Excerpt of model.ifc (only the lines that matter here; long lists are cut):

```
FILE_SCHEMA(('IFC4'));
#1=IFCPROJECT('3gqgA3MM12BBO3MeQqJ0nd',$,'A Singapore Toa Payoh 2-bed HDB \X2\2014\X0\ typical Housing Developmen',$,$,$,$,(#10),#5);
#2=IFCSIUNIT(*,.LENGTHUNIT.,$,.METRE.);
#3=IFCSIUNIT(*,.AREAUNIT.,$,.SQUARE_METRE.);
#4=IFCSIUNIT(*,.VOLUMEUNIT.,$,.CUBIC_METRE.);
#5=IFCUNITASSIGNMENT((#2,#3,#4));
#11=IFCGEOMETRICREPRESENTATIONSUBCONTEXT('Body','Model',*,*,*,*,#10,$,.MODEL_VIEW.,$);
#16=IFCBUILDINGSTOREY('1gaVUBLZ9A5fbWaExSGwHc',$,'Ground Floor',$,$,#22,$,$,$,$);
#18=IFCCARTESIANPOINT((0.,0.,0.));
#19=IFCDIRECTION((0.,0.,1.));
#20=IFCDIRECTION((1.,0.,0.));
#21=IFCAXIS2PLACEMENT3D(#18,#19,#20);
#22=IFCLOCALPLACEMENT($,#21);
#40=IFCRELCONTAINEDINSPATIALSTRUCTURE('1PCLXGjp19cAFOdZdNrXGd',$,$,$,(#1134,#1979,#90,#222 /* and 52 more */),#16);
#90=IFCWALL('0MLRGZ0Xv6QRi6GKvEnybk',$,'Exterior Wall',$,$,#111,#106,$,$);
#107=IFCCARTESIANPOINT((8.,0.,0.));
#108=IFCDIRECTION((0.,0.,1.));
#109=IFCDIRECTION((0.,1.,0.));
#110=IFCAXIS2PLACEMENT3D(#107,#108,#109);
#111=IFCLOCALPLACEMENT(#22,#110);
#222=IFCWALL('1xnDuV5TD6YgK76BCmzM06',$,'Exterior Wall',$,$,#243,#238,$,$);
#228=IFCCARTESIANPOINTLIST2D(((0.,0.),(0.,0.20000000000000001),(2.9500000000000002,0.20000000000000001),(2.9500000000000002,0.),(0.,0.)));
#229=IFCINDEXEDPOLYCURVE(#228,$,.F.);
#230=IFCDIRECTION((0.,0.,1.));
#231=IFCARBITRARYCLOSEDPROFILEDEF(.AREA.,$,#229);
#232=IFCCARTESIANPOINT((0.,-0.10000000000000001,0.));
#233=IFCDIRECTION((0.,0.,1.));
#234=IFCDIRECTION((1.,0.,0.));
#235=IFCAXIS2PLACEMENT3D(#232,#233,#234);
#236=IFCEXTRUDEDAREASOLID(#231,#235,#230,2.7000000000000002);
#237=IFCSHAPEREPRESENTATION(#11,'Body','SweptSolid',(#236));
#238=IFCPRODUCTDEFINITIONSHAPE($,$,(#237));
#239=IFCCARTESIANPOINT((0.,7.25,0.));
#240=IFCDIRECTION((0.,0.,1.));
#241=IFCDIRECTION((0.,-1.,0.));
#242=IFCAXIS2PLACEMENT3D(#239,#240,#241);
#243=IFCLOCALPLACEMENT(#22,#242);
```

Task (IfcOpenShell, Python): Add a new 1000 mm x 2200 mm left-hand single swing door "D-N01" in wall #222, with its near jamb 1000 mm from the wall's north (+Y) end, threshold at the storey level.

```python
import numpy as np
import ifcopenshell
import ifcopenshell.api.feature
import ifcopenshell.api.geometry
import ifcopenshell.api.root
import ifcopenshell.api.spatial
import ifcopenshell.geom
import ifcopenshell.util.element
import ifcopenshell.util.placement
import ifcopenshell.util.representation
import ifcopenshell.util.shape
import ifcopenshell.util.unit

model = ifcopenshell.open("model.ifc")
unit_scale = ifcopenshell.util.unit.calculate_unit_scale(model)
settings = ifcopenshell.geom.settings()


def volume(element):
    """Net volume in cubic metres, openings subtracted."""
    shape = ifcopenshell.geom.create_shape(settings, element)
    return ifcopenshell.util.shape.get_volume(shape.geometry)


wall = model.by_guid("1xnDuV5TD6YgK76BCmzM06")
storey = ifcopenshell.util.element.get_container(wall, ifc_class="IfcBuildingStorey")
context = ifcopenshell.util.representation.get_context(model, "Model", "Body", "MODEL_VIEW")
before = volume(wall)

width, height, from_end, sill = 1, 2.2, 1, 0.0  # metres

# The wall runs along its own X axis, and the end named is its -X end.
wall_shape = ifcopenshell.geom.create_shape(settings, wall)
x, y, z = ifcopenshell.util.shape.get_vertices(wall_shape.geometry).T
start = x.min() + from_end
face, thickness = float(y.min()), float(y.max() - y.min())
wall_matrix = ifcopenshell.util.placement.get_local_placement(wall.ObjectPlacement)
level = ifcopenshell.util.placement.get_local_placement(storey.ObjectPlacement)[2, 3]


def in_wall(x, y):
    """Placement at x, y metres in the wall's axes, at sill height."""
    matrix = wall_matrix.copy()
    matrix[:, 3] = wall_matrix @ np.array([x / unit_scale, y / unit_scale, 0.0, 1.0])
    matrix[2, 3] = level + sill / unit_scale
    return matrix


# Opening: a box that overshoots both wall faces by 50 mm.
opening = ifcopenshell.api.root.create_entity(model, ifc_class="IfcOpeningElement", predefined_type="OPENING")
box = ifcopenshell.api.geometry.add_wall_representation(
    model, context=context, length=width, height=height, thickness=thickness + 0.1
)
ifcopenshell.api.geometry.assign_representation(model, product=opening, representation=box)
ifcopenshell.api.geometry.edit_object_placement(model, product=opening, matrix=in_wall(start, face - 0.05), is_si=False)
ifcopenshell.api.feature.add_feature(model, feature=opening, element=wall)

door = ifcopenshell.api.root.create_entity(model, ifc_class="IfcDoor", name="D-N01", predefined_type="DOOR")
door.OverallWidth, door.OverallHeight = width / unit_scale, height / unit_scale
door.OperationType = "SINGLE_SWING_LEFT"
body = ifcopenshell.api.geometry.add_door_representation(
    model,
    context=context,
    overall_width=door.OverallWidth,
    overall_height=door.OverallHeight,
    operation_type="SINGLE_SWING_LEFT",
    lining_properties={"LiningDepth": thickness / unit_scale, "ThresholdDepth": thickness / unit_scale},
)
ifcopenshell.api.geometry.assign_representation(model, product=door, representation=body)
ifcopenshell.api.spatial.assign_container(model, products=[door], relating_structure=storey)
ifcopenshell.api.feature.add_filling(model, opening=opening, element=door)

# The lining spans the wall, so the door starts at the wall face.
ifcopenshell.api.geometry.edit_object_placement(model, product=door, matrix=in_wall(start, face), is_si=False)

after = volume(wall)

print(f"wall volume {before:.3f} -> {after:.3f} m3")

model.write("model-out.ifc")
```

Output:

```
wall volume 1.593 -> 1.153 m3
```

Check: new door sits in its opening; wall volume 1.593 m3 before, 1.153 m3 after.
